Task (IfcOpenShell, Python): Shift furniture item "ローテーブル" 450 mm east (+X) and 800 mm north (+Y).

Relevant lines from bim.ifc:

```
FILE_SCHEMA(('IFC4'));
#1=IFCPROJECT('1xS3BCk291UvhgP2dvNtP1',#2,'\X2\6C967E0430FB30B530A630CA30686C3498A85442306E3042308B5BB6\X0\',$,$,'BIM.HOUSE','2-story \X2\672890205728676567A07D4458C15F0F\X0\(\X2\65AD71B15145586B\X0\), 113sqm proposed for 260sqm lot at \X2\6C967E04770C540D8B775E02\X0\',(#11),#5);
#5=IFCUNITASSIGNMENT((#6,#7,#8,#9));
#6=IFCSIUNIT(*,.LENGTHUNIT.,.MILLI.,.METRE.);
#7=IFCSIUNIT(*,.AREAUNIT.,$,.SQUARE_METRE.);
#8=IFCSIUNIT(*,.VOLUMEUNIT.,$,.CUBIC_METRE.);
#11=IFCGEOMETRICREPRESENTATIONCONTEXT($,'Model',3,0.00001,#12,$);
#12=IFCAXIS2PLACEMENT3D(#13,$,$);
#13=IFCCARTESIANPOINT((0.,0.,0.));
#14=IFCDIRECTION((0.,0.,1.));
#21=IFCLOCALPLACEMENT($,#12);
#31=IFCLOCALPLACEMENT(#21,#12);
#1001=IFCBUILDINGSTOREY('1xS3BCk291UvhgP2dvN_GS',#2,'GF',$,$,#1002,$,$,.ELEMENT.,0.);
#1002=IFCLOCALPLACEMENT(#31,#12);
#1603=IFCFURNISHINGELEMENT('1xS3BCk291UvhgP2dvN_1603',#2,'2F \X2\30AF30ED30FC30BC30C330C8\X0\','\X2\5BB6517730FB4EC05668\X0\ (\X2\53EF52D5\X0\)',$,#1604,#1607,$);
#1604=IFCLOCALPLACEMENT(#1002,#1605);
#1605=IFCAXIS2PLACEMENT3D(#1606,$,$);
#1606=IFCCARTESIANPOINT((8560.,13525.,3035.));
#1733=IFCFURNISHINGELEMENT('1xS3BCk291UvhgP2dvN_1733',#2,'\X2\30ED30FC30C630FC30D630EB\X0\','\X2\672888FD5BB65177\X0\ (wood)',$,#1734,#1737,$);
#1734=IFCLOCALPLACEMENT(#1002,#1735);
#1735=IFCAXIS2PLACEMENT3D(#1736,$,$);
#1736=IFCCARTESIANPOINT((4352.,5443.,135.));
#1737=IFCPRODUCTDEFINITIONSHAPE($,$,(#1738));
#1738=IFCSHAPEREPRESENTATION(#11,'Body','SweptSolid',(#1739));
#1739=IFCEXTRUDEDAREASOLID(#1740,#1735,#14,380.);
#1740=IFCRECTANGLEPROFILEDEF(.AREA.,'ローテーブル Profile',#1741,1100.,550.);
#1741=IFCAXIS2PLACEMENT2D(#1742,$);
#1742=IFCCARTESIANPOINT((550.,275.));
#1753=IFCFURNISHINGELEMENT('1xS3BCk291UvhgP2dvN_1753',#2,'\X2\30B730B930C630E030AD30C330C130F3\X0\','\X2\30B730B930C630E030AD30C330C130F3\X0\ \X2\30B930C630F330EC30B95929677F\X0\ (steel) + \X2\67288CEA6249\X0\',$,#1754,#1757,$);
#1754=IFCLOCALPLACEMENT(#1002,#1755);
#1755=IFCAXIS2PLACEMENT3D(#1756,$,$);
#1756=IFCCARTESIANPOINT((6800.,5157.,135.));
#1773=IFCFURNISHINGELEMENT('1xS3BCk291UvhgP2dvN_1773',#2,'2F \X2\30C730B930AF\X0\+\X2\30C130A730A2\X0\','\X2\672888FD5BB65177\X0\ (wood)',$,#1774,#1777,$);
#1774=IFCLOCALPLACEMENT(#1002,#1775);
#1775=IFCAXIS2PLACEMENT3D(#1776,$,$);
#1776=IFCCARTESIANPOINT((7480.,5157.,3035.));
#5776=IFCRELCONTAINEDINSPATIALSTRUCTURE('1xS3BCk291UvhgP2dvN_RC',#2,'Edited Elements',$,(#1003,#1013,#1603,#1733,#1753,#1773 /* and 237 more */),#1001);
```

```python
import ifcopenshell
import ifcopenshell.api.geometry
import ifcopenshell.util.placement
import ifcopenshell.util.unit

model = ifcopenshell.open("bim.ifc")
unit_scale = ifcopenshell.util.unit.calculate_unit_scale(model)

item = model.by_guid("1xS3BCk291UvhgP2dvN_1733")
matrix = ifcopenshell.util.placement.get_local_placement(item.ObjectPlacement)
matrix[0, 3] += 0.45 / unit_scale
matrix[1, 3] += 0.8 / unit_scale
ifcopenshell.api.geometry.edit_object_placement(model, product=item, matrix=matrix, is_si=False)

print(ifcopenshell.util.placement.get_local_placement(item.ObjectPlacement).round(3) + 0.0)

model.write("bim-out.ifc")
```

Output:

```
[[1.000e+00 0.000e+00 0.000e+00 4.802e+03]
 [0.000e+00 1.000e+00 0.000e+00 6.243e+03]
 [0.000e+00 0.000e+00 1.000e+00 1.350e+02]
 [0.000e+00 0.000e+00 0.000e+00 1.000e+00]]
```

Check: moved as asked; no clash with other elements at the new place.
